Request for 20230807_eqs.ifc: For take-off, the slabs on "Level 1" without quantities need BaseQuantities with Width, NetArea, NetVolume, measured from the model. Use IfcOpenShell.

First a look at what the model holds.

```python
import ifcopenshell
import ifcopenshell.util.element
import ifcopenshell.util.unit

model = ifcopenshell.open("20230807_eqs.ifc")
print(model.schema)
for unit_type in ("LENGTHUNIT", "AREAUNIT", "VOLUMEUNIT"):
    print(unit_type, ifcopenshell.util.unit.calculate_unit_scale(model, unit_type))
storey = next(s for s in model.by_type("IfcBuildingStorey") if s.Name == "Level 1")
slabs = [e for e in ifcopenshell.util.element.get_decomposition(storey) if e.is_a("IfcSlab")]
for e in sorted(slabs, key=lambda e: e.id()):
    print(e.id(), e.is_a(), e.Name, list(ifcopenshell.util.element.get_psets(e, qtos_only=True)), sep=" | ")
```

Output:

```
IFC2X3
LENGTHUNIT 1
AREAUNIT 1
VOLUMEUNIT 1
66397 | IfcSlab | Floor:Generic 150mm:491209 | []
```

```python
import ifcopenshell
import ifcopenshell.api.pset
import ifcopenshell.geom
import ifcopenshell.util.element
import ifcopenshell.util.shape
import ifcopenshell.util.unit

model = ifcopenshell.open("20230807_eqs.ifc")
unit_scale = ifcopenshell.util.unit.calculate_unit_scale(model)
area_scale = ifcopenshell.util.unit.calculate_unit_scale(model, "AREAUNIT")
volume_scale = ifcopenshell.util.unit.calculate_unit_scale(model, "VOLUMEUNIT")
settings = ifcopenshell.geom.settings()

storey = next(s for s in model.by_type("IfcBuildingStorey") if s.Name == "Level 1")
slabs = [e for e in ifcopenshell.util.element.get_decomposition(storey) if e.is_a("IfcSlab")]

for e in sorted(slabs, key=lambda e: e.id()):
    if ifcopenshell.util.element.get_psets(e, qtos_only=True, should_inherit=False):
        continue
    # Geometry comes back in metres, in the element's own axes.
    shape = ifcopenshell.geom.create_shape(settings, e)
    values = {
        "Width": ifcopenshell.util.shape.get_z(shape.geometry) / unit_scale,
        "NetArea": ifcopenshell.util.shape.get_footprint_area(shape.geometry) / area_scale,
        "NetVolume": ifcopenshell.util.shape.get_volume(shape.geometry) / volume_scale,
    }
    qto = ifcopenshell.api.pset.add_qto(model, product=e, name="BaseQuantities")
    ifcopenshell.api.pset.edit_qto(model, qto=qto, properties=values)
    print(e.id(), {k: round(v, 3) for k, v in values.items()})

model.write("20230807_eqs_updated.ifc")
```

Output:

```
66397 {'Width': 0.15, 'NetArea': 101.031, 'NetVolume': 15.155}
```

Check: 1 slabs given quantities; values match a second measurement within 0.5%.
